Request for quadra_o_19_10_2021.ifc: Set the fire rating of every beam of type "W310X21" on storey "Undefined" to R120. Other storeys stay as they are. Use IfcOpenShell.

First a look at what the model holds.

```python
import ifcopenshell
import ifcopenshell.util.element

model = ifcopenshell.open("quadra_o_19_10_2021.ifc")
print(model.schema)
storey = next(s for s in model.by_type("IfcBuildingStorey") if s.Name == "Undefined")
beams = [e for e in ifcopenshell.util.element.get_decomposition(storey) if e.is_a("IfcBeam")]
seen = {}
for e in beams:
    element_type = ifcopenshell.util.element.get_type(e)
    key = (element_type.Name if element_type != e and element_type else None, ifcopenshell.util.element.get_pset(e, "Pset_BeamCommon", "FireRating"))
    seen[key] = seen.get(key, 0) + 1
for (name, value), count in sorted(seen.items(), key=str):
    print(count, "x", name, "|", value)
```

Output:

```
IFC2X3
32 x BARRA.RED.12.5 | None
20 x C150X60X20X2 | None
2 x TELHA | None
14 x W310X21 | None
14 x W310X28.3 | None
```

```python
import ifcopenshell
import ifcopenshell.api.pset
import ifcopenshell.util.element

model = ifcopenshell.open("quadra_o_19_10_2021.ifc")

storey = next(s for s in model.by_type("IfcBuildingStorey") if s.Name == "Undefined")
beams = [e for e in ifcopenshell.util.element.get_decomposition(storey) if e.is_a("IfcBeam")]

count = 0
for e in beams:
    element_type = ifcopenshell.util.element.get_type(e)
    if element_type in (None, e) or element_type.Name != "W310X21":
        continue
    found = ifcopenshell.util.element.get_pset(e, "Pset_BeamCommon", should_inherit=False)
    if found:
        pset = model.by_id(found["id"])
        if len(ifcopenshell.util.element.get_elements_by_pset(pset)) > 1:
            pset = ifcopenshell.api.pset.unshare_pset(model, products=[e], pset=pset)[0]
    else:
        pset = ifcopenshell.api.pset.add_pset(model, product=e, name="Pset_BeamCommon")
    ifcopenshell.api.pset.edit_pset(model, pset=pset, properties={"FireRating": "R120"})
    count += 1

print(count, "beams updated")

model.write("quadra_o_19_10_2021_edited.ifc")
```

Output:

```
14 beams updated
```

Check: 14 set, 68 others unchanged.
